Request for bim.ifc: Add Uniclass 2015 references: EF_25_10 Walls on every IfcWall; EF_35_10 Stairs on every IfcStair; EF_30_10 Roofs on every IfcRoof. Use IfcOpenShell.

First a look at what the model holds.

```python
import ifcopenshell

model = ifcopenshell.open("bim.ifc")
print(model.schema)
print("classifications:", [c.Name for c in model.by_type("IfcClassification")])
for ifc_class in ("IfcDoor", "IfcRoof", "IfcStair", "IfcWall", "IfcWindow"):
    print(ifc_class, len(model.by_type(ifc_class)))
```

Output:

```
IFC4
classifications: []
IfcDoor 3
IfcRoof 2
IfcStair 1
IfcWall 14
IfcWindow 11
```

```python
import ifcopenshell
import ifcopenshell.api.classification

model = ifcopenshell.open("bim.ifc")

system = ifcopenshell.api.classification.add_classification(model, classification="Uniclass 2015")

codes = {
    "IfcWall": ("EF_25_10", "Walls"),
    "IfcStair": ("EF_35_10", "Stairs"),
    "IfcRoof": ("EF_30_10", "Roofs"),
}
for ifc_class, (code, name) in codes.items():
    products = model.by_type(ifc_class)
    ifcopenshell.api.classification.add_reference(
        model, products=products, classification=system, identification=code, name=name
    )
    print(code, len(products))

model.write("bim_edited.ifc")
```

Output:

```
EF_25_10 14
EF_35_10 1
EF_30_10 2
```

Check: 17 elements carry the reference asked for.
